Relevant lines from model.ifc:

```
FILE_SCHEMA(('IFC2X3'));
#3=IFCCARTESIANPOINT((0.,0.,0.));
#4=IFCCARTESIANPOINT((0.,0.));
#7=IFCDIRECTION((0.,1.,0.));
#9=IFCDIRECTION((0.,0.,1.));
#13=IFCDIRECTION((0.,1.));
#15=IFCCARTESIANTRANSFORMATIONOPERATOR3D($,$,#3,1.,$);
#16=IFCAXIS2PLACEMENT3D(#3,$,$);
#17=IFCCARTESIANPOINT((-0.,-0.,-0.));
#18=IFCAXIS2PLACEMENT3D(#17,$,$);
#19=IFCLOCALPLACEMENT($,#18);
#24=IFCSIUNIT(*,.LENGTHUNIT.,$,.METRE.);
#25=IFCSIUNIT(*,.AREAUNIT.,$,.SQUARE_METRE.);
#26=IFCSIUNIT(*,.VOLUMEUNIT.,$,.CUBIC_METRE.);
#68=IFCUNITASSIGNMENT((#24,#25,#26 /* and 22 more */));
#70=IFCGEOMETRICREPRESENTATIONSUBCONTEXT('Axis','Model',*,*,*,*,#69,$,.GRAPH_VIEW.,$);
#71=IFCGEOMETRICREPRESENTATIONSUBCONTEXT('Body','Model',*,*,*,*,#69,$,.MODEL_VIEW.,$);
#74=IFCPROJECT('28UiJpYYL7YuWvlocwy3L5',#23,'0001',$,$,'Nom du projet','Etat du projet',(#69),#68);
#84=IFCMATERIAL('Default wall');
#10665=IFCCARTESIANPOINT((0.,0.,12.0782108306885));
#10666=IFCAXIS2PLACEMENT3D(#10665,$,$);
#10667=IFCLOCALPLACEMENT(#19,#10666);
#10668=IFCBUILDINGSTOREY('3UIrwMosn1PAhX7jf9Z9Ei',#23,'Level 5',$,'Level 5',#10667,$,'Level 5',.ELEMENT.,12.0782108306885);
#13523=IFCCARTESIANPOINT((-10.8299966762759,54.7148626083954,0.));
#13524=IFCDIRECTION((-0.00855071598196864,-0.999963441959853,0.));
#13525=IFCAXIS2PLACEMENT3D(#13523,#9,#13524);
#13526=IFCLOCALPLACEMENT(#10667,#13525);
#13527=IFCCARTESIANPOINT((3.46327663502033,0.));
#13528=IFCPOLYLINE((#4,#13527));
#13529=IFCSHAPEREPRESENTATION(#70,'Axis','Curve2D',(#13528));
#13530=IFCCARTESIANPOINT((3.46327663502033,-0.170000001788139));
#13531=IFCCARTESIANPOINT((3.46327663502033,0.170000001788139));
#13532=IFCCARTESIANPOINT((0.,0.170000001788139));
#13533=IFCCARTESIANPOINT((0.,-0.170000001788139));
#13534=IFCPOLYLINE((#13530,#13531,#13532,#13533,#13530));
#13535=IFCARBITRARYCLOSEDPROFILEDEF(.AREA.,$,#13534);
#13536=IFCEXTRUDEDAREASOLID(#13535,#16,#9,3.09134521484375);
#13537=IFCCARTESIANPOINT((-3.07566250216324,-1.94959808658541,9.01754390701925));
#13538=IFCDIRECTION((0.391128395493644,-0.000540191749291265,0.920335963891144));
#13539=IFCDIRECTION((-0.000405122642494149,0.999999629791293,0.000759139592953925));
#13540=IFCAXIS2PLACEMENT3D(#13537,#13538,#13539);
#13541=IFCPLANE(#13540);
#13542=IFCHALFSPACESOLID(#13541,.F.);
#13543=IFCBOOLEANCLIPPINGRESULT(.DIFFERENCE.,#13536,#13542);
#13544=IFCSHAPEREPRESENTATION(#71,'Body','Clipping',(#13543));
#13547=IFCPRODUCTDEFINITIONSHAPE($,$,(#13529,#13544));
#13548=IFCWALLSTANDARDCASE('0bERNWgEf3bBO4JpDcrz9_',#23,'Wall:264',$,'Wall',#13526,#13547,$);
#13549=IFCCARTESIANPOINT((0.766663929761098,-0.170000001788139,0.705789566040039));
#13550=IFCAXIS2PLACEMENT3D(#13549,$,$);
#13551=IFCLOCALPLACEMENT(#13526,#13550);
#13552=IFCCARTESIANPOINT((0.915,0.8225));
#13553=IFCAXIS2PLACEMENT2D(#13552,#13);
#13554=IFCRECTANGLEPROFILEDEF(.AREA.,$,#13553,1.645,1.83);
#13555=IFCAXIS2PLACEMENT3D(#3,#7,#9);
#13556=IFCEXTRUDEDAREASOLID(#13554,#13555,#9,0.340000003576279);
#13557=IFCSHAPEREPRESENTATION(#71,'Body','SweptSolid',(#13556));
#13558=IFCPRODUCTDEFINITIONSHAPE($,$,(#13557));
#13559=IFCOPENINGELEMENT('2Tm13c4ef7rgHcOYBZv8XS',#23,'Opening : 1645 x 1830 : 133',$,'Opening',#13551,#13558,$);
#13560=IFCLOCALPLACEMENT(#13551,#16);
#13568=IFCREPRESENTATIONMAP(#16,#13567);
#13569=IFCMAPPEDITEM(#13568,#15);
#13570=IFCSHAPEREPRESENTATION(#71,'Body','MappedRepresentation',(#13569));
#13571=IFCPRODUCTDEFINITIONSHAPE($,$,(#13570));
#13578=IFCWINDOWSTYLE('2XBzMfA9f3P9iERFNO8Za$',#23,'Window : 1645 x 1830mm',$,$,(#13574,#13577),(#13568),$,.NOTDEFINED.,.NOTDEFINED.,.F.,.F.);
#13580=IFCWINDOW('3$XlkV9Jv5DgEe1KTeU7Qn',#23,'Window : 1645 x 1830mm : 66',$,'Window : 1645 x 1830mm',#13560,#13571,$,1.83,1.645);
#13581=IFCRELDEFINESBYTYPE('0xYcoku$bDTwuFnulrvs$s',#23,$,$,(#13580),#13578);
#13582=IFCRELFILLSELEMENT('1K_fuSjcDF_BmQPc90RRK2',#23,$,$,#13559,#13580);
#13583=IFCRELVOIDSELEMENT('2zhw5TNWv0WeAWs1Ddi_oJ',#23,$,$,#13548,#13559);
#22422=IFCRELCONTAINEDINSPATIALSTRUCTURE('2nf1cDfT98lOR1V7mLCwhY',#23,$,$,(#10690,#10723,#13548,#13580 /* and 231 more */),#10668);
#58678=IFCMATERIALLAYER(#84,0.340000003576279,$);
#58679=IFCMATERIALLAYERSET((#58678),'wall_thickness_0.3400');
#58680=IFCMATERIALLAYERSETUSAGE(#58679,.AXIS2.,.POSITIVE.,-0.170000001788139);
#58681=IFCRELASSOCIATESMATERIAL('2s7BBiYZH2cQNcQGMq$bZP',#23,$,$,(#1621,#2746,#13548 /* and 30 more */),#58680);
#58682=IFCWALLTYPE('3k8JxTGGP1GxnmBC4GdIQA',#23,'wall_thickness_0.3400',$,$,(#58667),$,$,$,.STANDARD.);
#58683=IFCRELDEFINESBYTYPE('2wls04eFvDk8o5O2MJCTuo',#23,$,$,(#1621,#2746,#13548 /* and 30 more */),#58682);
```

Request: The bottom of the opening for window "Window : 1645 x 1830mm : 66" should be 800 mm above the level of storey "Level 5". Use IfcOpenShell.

```python
import numpy as np
import ifcopenshell
import ifcopenshell.api.geometry
import ifcopenshell.geom
import ifcopenshell.util.element
import ifcopenshell.util.placement
import ifcopenshell.util.shape
import ifcopenshell.util.unit

model = ifcopenshell.open("model.ifc")
unit_scale = ifcopenshell.util.unit.calculate_unit_scale(model)

window = model.by_guid("3$XlkV9Jv5DgEe1KTeU7Qn")
opening = window.FillsVoids[0].RelatingOpeningElement
storey = ifcopenshell.util.element.get_container(window, ifc_class="IfcBuildingStorey")
level = ifcopenshell.util.placement.get_local_placement(storey.ObjectPlacement)[2, 3]

# The opening's origin need not be at the sill, so measure its lowest point.
shape = ifcopenshell.geom.create_shape(ifcopenshell.geom.settings(), opening)
bottom = ifcopenshell.util.shape.get_shape_bottom_elevation(shape, shape.geometry) / unit_scale
dz = level + 0.8 / unit_scale - bottom

shift = np.array([0.0, 0.0, dz])
# The window is placed relative to its opening, so it follows when the opening moves.
matrix = ifcopenshell.util.placement.get_local_placement(opening.ObjectPlacement)
matrix[:3, 3] += shift
ifcopenshell.api.geometry.edit_object_placement(
    model, product=opening, matrix=matrix, is_si=False, should_transform_children=True
)

print(f"moved by {dz * unit_scale:+.3f} m")

model.write("model-out.ifc")
```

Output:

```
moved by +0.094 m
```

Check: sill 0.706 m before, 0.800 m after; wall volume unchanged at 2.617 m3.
